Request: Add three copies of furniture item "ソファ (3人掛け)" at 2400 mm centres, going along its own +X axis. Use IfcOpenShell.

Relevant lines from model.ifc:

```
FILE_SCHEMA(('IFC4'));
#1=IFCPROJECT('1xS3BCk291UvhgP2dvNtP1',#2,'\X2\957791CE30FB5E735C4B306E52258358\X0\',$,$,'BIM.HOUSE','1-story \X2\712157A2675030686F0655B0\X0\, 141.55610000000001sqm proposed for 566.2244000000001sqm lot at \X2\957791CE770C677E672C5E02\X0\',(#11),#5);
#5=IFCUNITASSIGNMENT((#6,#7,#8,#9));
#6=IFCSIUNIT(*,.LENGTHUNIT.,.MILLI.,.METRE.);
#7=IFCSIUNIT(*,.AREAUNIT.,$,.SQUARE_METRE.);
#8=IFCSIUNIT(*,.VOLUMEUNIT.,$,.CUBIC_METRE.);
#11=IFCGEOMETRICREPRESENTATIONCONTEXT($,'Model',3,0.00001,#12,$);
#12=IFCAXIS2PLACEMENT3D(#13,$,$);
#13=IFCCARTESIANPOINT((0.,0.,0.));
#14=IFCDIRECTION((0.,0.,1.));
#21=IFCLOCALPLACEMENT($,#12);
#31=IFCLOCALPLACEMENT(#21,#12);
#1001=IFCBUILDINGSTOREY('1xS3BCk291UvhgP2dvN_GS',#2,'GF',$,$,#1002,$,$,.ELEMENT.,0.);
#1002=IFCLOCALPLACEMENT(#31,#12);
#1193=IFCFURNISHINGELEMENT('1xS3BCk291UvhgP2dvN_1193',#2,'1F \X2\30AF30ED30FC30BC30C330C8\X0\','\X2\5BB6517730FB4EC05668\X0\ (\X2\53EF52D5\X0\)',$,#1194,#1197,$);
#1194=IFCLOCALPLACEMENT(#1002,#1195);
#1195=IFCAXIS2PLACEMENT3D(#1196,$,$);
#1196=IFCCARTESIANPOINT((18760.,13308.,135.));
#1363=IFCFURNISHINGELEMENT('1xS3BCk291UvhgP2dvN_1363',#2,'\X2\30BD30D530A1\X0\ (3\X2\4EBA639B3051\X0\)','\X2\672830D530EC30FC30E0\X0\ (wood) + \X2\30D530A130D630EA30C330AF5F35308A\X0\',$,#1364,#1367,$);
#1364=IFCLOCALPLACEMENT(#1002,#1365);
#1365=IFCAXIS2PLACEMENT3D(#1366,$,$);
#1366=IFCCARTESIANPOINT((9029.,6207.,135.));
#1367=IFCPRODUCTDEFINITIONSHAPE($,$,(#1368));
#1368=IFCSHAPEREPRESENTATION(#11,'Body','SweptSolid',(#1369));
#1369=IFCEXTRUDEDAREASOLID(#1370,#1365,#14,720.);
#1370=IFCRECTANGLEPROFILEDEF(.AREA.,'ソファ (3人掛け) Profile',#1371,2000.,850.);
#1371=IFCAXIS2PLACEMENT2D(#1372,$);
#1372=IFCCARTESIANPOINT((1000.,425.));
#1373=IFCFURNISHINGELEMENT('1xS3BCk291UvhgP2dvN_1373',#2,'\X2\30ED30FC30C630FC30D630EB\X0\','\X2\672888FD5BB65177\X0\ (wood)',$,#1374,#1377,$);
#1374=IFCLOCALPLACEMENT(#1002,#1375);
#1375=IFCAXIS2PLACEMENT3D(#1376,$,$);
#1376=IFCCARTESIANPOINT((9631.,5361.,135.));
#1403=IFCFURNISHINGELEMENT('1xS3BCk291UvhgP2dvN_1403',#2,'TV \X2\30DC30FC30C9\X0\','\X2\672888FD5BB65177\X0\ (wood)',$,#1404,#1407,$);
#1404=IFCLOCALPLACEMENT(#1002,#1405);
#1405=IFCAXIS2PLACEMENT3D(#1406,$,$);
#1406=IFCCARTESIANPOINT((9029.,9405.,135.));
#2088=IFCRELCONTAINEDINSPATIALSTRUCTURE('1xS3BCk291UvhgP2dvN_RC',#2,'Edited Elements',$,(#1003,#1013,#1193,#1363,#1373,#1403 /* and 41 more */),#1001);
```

```python
import ifcopenshell
import ifcopenshell.api.geometry
import ifcopenshell.api.root
import ifcopenshell.util.element
import ifcopenshell.util.placement

model = ifcopenshell.open("model.ifc")


def reuse_history(source, copy):
    """copy_class also copies each property set's owner history, people and application; keep the originals."""
    for rel in copy.IsDefinedBy:
        if rel.is_a("IfcRelDefinesByProperties") and (history := rel.RelatingPropertyDefinition.OwnerHistory):
            rel.RelatingPropertyDefinition.OwnerHistory = source.OwnerHistory
            ifcopenshell.util.element.remove_deep2(model, history)


source = model.by_guid("1xS3BCk291UvhgP2dvN_1363")
base = ifcopenshell.util.placement.get_local_placement(source.ObjectPlacement)
step = base[:3, 0] * 2400.0

for i in range(1, 4):
    copy = ifcopenshell.api.root.copy_class(model, product=source)
    copy.Representation = ifcopenshell.util.element.copy_deep(
        model, source.Representation, exclude=["IfcGeometricRepresentationContext", "IfcRepresentationMap"]
    )
    reuse_history(source, copy)
    matrix = base.copy()
    matrix[:3, 3] += i * step
    print("added at", matrix[:3, 3].round(3) + 0.0)
    ifcopenshell.api.geometry.edit_object_placement(model, product=copy, matrix=matrix, is_si=False)

model.write("model_v2.ifc")
```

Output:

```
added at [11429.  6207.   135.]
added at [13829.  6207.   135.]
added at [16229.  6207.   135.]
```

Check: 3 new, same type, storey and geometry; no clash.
